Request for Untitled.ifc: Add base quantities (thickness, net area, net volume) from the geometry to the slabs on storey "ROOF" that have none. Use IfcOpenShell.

First a look at what the model holds.

```python
import ifcopenshell
import ifcopenshell.util.element
import ifcopenshell.util.unit

model = ifcopenshell.open("Untitled.ifc")
print(model.schema)
for unit_type in ("LENGTHUNIT", "AREAUNIT", "VOLUMEUNIT"):
    print(unit_type, ifcopenshell.util.unit.calculate_unit_scale(model, unit_type))
storey = next(s for s in model.by_type("IfcBuildingStorey") if s.Name == "ROOF")
slabs = [e for e in ifcopenshell.util.element.get_decomposition(storey) if e.is_a("IfcSlab")]
for e in sorted(slabs, key=lambda e: e.id()):
    print(e.id(), e.is_a(), e.Name, list(ifcopenshell.util.element.get_psets(e, qtos_only=True)), sep=" | ")
```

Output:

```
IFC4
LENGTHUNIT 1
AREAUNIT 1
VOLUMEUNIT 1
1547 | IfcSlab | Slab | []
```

```python
import ifcopenshell
import ifcopenshell.api.pset
import ifcopenshell.geom
import ifcopenshell.util.element
import ifcopenshell.util.shape
import ifcopenshell.util.unit

model = ifcopenshell.open("Untitled.ifc")
unit_scale = ifcopenshell.util.unit.calculate_unit_scale(model)
area_scale = ifcopenshell.util.unit.calculate_unit_scale(model, "AREAUNIT")
volume_scale = ifcopenshell.util.unit.calculate_unit_scale(model, "VOLUMEUNIT")
settings = ifcopenshell.geom.settings()

storey = next(s for s in model.by_type("IfcBuildingStorey") if s.Name == "ROOF")
slabs = [e for e in ifcopenshell.util.element.get_decomposition(storey) if e.is_a("IfcSlab")]

for e in sorted(slabs, key=lambda e: e.id()):
    if ifcopenshell.util.element.get_psets(e, qtos_only=True, should_inherit=False):
        continue
    # Geometry comes back in metres, in the element's own axes.
    shape = ifcopenshell.geom.create_shape(settings, e)
    values = {
        "Width": ifcopenshell.util.shape.get_z(shape.geometry) / unit_scale,
        "NetArea": ifcopenshell.util.shape.get_footprint_area(shape.geometry) / area_scale,
        "NetVolume": ifcopenshell.util.shape.get_volume(shape.geometry) / volume_scale,
    }
    qto = ifcopenshell.api.pset.add_qto(model, product=e, name="Qto_SlabBaseQuantities")
    ifcopenshell.api.pset.edit_qto(model, qto=qto, properties=values)
    print(e.id(), {k: round(v, 3) for k, v in values.items()})

model.write("Untitled_rev.ifc")
```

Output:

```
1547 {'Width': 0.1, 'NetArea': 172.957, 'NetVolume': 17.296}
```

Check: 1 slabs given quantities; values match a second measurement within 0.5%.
